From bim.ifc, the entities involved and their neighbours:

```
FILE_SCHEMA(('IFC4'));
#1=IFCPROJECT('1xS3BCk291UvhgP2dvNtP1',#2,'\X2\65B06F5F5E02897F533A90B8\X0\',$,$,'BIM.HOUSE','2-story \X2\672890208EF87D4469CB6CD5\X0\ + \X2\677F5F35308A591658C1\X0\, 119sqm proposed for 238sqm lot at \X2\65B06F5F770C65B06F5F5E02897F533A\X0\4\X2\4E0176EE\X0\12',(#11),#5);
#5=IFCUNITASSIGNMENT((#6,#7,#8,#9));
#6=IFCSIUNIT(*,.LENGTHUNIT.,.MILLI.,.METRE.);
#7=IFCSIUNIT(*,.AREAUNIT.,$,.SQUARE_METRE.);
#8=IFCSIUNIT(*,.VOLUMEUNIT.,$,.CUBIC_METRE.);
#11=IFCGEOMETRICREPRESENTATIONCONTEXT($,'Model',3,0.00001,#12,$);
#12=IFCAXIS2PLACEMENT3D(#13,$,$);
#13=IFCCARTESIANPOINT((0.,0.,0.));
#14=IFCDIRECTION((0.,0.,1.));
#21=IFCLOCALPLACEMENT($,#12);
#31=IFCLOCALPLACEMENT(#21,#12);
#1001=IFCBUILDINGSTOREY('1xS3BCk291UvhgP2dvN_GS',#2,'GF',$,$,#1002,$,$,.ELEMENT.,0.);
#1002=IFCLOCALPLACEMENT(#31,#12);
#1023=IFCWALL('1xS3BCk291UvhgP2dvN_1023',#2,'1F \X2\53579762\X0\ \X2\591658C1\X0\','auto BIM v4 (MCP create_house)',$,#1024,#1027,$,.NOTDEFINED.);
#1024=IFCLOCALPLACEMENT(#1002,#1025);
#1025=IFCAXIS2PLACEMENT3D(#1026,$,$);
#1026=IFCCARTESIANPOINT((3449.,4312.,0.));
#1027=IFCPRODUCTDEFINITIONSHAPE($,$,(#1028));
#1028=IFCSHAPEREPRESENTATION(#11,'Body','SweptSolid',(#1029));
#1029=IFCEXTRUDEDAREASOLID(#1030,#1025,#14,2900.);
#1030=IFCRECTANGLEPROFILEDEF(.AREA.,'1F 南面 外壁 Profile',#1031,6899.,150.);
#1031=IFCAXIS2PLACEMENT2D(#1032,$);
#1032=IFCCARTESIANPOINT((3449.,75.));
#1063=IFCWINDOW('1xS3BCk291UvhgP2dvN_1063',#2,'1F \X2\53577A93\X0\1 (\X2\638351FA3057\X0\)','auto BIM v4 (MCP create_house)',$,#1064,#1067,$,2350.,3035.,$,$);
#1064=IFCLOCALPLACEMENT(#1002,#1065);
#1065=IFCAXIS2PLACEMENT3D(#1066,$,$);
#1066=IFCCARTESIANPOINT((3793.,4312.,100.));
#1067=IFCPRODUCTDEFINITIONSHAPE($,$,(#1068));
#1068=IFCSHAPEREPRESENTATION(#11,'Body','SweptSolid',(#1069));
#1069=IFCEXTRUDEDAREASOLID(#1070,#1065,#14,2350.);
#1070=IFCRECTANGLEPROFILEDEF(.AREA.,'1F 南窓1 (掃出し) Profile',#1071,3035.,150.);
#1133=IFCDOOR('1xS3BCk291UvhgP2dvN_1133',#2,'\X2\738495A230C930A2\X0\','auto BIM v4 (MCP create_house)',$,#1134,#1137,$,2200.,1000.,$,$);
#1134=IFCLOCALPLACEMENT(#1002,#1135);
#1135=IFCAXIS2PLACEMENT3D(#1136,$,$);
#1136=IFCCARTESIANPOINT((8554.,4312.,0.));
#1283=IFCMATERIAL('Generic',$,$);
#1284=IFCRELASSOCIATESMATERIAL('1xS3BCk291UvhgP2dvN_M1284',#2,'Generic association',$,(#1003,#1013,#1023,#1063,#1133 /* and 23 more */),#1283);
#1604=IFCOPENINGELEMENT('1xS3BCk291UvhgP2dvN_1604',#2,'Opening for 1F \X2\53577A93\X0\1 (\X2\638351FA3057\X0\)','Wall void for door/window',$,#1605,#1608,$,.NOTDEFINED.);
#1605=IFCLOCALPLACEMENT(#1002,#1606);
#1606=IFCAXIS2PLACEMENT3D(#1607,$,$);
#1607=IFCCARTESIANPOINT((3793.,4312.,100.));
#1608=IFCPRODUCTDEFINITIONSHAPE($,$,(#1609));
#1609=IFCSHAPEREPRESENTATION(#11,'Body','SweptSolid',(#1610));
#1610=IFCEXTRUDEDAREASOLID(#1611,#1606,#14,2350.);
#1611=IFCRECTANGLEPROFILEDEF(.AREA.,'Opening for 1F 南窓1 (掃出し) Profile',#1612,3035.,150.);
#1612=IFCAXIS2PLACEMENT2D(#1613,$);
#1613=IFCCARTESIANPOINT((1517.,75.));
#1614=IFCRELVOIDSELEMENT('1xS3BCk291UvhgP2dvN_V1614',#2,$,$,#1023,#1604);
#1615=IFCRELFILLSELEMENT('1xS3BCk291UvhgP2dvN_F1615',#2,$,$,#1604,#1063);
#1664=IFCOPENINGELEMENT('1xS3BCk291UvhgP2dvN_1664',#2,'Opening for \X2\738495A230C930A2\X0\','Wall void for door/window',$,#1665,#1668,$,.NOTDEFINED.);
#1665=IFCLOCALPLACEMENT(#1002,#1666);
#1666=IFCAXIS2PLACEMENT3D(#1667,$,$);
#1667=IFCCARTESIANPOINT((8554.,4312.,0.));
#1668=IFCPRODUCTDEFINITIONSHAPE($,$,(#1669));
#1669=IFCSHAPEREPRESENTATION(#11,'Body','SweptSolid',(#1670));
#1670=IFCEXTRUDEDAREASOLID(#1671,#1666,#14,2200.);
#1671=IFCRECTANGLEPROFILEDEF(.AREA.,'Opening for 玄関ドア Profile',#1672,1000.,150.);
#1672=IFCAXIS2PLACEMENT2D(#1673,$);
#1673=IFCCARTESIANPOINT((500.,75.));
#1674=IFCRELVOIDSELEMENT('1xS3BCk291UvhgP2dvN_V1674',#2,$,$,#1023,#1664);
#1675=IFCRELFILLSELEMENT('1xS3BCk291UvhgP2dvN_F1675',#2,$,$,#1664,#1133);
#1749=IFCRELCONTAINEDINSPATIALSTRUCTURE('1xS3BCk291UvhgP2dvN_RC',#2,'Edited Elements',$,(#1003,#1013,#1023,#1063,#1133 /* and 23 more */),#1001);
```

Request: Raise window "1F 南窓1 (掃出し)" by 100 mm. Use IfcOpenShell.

```python
import numpy as np
import ifcopenshell
import ifcopenshell.api.geometry
import ifcopenshell.util.placement
import ifcopenshell.util.unit

model = ifcopenshell.open("bim.ifc")
unit_scale = ifcopenshell.util.unit.calculate_unit_scale(model)

window = model.by_id(1063)
opening = window.FillsVoids[0].RelatingOpeningElement
dz = 100.0

shift = np.array([0.0, 0.0, dz])
# The window is not placed relative to its opening, so move both.
for product in (opening, window):
    matrix = ifcopenshell.util.placement.get_local_placement(product.ObjectPlacement)
    matrix[:3, 3] += shift
    ifcopenshell.api.geometry.edit_object_placement(model, product=product, matrix=matrix, is_si=False)

print(f"moved by {dz * unit_scale:+.3f} m")

model.write("bim-out.ifc")
```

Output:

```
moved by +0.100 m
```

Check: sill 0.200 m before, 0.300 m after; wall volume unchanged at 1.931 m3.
